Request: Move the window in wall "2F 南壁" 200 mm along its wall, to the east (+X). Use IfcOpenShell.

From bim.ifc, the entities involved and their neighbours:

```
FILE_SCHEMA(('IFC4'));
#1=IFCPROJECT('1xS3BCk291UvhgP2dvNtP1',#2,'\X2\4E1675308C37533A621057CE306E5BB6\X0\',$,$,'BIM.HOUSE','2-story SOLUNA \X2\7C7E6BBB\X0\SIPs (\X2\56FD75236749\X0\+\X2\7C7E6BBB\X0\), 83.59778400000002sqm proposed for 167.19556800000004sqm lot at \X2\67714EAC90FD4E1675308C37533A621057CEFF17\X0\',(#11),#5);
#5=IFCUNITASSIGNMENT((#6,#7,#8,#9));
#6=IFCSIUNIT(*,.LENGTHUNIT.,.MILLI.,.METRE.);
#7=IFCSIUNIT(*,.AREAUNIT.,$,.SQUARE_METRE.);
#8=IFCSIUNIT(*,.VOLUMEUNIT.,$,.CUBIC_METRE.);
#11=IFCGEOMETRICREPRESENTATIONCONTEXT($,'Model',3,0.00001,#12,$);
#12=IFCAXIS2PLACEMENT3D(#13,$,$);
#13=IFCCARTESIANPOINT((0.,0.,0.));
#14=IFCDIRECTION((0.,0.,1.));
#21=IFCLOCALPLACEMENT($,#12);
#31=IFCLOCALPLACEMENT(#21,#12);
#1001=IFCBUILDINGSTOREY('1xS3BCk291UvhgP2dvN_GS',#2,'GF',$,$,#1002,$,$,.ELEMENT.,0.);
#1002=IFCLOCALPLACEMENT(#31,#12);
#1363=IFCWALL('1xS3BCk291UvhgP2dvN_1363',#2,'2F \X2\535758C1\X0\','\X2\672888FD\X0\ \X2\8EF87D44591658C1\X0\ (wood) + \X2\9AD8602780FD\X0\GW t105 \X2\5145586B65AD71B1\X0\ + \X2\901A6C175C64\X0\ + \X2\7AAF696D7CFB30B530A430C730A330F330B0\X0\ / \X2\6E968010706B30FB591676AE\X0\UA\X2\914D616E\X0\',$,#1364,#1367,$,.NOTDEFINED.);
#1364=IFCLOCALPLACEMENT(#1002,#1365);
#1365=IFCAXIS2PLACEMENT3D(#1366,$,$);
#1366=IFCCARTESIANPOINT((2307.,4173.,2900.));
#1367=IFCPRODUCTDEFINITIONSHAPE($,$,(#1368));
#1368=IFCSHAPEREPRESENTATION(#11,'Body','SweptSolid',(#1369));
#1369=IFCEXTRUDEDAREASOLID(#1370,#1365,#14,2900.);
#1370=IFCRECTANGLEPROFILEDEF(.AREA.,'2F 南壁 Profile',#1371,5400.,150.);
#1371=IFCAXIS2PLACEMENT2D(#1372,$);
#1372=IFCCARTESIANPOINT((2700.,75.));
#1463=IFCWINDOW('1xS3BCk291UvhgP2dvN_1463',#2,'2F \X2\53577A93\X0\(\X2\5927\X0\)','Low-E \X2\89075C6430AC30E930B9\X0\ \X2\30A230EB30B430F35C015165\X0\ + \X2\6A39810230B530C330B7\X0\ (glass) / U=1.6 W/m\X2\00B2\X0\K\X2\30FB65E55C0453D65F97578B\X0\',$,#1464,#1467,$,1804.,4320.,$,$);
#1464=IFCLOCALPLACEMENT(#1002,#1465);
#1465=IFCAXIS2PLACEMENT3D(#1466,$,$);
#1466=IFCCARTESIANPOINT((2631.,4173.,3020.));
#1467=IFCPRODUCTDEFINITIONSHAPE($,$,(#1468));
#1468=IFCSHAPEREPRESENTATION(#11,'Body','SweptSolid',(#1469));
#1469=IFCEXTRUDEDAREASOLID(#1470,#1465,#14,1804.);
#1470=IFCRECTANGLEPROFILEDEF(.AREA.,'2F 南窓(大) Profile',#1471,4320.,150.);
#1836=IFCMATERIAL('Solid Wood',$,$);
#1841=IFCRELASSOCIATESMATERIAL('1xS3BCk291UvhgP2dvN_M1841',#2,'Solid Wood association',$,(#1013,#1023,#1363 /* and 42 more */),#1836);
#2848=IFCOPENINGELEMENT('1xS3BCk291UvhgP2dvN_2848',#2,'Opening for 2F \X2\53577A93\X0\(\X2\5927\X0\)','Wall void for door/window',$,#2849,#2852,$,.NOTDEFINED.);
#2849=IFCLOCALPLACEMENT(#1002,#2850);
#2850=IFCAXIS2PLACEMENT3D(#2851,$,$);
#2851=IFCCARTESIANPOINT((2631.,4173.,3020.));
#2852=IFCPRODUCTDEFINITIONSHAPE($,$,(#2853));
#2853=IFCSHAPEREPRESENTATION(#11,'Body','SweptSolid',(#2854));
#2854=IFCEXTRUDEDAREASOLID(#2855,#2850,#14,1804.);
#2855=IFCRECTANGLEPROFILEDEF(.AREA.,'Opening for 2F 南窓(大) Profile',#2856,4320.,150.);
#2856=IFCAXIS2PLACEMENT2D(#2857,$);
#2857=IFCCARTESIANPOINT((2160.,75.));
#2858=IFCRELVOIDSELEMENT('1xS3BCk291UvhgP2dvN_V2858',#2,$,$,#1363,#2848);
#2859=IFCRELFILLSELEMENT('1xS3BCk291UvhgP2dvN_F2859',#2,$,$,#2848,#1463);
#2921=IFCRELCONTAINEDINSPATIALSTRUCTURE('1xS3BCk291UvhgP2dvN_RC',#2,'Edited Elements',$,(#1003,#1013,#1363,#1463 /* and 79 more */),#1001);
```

```python
import ifcopenshell
import ifcopenshell.api.geometry
import ifcopenshell.util.placement

model = ifcopenshell.open("bim.ifc")

window = model.by_guid("1xS3BCk291UvhgP2dvN_1463")
opening = window.FillsVoids[0].RelatingOpeningElement
wall = opening.VoidsElements[0].RelatingBuildingElement

wall_matrix = ifcopenshell.util.placement.get_local_placement(wall.ObjectPlacement)
shift = wall_matrix[:3, 0] * 200.0
before = ifcopenshell.util.placement.get_local_placement(window.ObjectPlacement)[:3, 3].copy()

# The window is not placed relative to its opening, so move both.
for product in (opening, window):
    matrix = ifcopenshell.util.placement.get_local_placement(product.ObjectPlacement)
    matrix[:3, 3] += shift
    ifcopenshell.api.geometry.edit_object_placement(model, product=product, matrix=matrix, is_si=False)

after = ifcopenshell.util.placement.get_local_placement(window.ObjectPlacement)[:3, 3]
print("window moved by", (after - before).round(3) + 0.0)

model.write("bim_v2.ifc")
```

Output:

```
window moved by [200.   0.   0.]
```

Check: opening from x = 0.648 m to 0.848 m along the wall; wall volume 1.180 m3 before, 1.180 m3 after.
